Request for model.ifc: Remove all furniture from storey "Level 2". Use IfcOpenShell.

First a look at what the model holds.

```python
import ifcopenshell
import ifcopenshell.util.element

model = ifcopenshell.open("model.ifc")
print(model.schema)
storey = next(s for s in model.by_type("IfcBuildingStorey") if s.Name == "Level 2")
furniture = [e for e in ifcopenshell.util.element.get_decomposition(storey) if e.is_a("IfcFurnishingElement")]
seen = {}
for e in furniture:
    element_type = ifcopenshell.util.element.get_type(e)
    name = element_type.Name if element_type not in (None, e) else None
    seen[name] = seen.get(name, 0) + 1
for name, count in sorted(seen.items(), key=str):
    print(count, "x", name)
```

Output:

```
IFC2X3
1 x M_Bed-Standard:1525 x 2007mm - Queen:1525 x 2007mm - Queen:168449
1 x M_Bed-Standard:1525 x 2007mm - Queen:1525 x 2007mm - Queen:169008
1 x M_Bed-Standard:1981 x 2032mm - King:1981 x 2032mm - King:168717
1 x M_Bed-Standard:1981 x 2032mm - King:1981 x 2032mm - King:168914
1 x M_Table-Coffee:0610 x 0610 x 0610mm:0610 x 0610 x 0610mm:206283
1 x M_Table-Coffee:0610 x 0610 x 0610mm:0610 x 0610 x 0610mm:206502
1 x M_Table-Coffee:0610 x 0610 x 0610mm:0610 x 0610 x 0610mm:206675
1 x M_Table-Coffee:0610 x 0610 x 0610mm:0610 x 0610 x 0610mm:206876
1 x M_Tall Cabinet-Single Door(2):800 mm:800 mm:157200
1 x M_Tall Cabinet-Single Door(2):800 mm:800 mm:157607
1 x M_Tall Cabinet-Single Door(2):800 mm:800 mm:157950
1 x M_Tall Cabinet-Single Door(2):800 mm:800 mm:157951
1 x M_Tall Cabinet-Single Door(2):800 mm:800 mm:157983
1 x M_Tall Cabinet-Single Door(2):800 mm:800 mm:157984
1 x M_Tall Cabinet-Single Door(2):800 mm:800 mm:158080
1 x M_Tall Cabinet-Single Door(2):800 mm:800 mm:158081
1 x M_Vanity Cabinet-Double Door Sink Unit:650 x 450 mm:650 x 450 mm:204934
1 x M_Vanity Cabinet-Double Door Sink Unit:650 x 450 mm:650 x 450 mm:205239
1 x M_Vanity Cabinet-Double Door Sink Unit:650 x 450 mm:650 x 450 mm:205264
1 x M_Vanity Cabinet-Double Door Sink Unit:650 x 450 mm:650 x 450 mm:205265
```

```python
import ifcopenshell
import ifcopenshell.api.root
import ifcopenshell.util.element

model = ifcopenshell.open("model.ifc")

storey = next(s for s in model.by_type("IfcBuildingStorey") if s.Name == "Level 2")
furniture = [e for e in ifcopenshell.util.element.get_decomposition(storey) if e.is_a("IfcFurnishingElement")]

for e in furniture:
    ifcopenshell.api.root.remove_product(model, product=e)
print(len(furniture), "removed")

model.write("model_v2.ifc")
```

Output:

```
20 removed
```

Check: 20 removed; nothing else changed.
